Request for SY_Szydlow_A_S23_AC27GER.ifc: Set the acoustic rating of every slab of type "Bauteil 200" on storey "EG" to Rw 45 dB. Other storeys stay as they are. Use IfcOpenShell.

First a look at what the model holds.

```python
import ifcopenshell
import ifcopenshell.util.element

model = ifcopenshell.open("SY_Szydlow_A_S23_AC27GER.ifc")
print(model.schema)
storey = next(s for s in model.by_type("IfcBuildingStorey") if s.Name == "EG")
slabs = [e for e in ifcopenshell.util.element.get_decomposition(storey) if e.is_a("IfcSlab")]
seen = {}
for e in slabs:
    element_type = ifcopenshell.util.element.get_type(e)
    key = (element_type.Name if element_type != e and element_type else None, ifcopenshell.util.element.get_pset(e, "Pset_SlabCommon", "AcousticRating"))
    seen[key] = seen.get(key, 0) + 1
for (name, value), count in sorted(seen.items(), key=str):
    print(count, "x", name, "|", value)
```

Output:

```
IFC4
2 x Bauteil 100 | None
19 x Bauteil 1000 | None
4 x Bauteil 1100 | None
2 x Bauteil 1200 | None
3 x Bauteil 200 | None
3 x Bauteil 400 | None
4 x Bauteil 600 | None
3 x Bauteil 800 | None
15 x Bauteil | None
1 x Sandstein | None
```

```python
import ifcopenshell
import ifcopenshell.api.pset
import ifcopenshell.util.element

model = ifcopenshell.open("SY_Szydlow_A_S23_AC27GER.ifc")

storey = next(s for s in model.by_type("IfcBuildingStorey") if s.Name == "EG")
slabs = [e for e in ifcopenshell.util.element.get_decomposition(storey) if e.is_a("IfcSlab")]

count = 0
for e in slabs:
    element_type = ifcopenshell.util.element.get_type(e)
    if element_type in (None, e) or element_type.Name != "Bauteil 200":
        continue
    # add_pset returns the element's existing set when there is one.
    pset = ifcopenshell.api.pset.add_pset(model, product=e, name="Pset_SlabCommon")
    ifcopenshell.api.pset.edit_pset(model, pset=pset, properties={"AcousticRating": "Rw 45 dB"})
    count += 1

print(count, "slabs updated")

model.write("SY_Szydlow_A_S23_AC27GER_rev.ifc")
```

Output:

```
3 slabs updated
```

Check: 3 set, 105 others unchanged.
